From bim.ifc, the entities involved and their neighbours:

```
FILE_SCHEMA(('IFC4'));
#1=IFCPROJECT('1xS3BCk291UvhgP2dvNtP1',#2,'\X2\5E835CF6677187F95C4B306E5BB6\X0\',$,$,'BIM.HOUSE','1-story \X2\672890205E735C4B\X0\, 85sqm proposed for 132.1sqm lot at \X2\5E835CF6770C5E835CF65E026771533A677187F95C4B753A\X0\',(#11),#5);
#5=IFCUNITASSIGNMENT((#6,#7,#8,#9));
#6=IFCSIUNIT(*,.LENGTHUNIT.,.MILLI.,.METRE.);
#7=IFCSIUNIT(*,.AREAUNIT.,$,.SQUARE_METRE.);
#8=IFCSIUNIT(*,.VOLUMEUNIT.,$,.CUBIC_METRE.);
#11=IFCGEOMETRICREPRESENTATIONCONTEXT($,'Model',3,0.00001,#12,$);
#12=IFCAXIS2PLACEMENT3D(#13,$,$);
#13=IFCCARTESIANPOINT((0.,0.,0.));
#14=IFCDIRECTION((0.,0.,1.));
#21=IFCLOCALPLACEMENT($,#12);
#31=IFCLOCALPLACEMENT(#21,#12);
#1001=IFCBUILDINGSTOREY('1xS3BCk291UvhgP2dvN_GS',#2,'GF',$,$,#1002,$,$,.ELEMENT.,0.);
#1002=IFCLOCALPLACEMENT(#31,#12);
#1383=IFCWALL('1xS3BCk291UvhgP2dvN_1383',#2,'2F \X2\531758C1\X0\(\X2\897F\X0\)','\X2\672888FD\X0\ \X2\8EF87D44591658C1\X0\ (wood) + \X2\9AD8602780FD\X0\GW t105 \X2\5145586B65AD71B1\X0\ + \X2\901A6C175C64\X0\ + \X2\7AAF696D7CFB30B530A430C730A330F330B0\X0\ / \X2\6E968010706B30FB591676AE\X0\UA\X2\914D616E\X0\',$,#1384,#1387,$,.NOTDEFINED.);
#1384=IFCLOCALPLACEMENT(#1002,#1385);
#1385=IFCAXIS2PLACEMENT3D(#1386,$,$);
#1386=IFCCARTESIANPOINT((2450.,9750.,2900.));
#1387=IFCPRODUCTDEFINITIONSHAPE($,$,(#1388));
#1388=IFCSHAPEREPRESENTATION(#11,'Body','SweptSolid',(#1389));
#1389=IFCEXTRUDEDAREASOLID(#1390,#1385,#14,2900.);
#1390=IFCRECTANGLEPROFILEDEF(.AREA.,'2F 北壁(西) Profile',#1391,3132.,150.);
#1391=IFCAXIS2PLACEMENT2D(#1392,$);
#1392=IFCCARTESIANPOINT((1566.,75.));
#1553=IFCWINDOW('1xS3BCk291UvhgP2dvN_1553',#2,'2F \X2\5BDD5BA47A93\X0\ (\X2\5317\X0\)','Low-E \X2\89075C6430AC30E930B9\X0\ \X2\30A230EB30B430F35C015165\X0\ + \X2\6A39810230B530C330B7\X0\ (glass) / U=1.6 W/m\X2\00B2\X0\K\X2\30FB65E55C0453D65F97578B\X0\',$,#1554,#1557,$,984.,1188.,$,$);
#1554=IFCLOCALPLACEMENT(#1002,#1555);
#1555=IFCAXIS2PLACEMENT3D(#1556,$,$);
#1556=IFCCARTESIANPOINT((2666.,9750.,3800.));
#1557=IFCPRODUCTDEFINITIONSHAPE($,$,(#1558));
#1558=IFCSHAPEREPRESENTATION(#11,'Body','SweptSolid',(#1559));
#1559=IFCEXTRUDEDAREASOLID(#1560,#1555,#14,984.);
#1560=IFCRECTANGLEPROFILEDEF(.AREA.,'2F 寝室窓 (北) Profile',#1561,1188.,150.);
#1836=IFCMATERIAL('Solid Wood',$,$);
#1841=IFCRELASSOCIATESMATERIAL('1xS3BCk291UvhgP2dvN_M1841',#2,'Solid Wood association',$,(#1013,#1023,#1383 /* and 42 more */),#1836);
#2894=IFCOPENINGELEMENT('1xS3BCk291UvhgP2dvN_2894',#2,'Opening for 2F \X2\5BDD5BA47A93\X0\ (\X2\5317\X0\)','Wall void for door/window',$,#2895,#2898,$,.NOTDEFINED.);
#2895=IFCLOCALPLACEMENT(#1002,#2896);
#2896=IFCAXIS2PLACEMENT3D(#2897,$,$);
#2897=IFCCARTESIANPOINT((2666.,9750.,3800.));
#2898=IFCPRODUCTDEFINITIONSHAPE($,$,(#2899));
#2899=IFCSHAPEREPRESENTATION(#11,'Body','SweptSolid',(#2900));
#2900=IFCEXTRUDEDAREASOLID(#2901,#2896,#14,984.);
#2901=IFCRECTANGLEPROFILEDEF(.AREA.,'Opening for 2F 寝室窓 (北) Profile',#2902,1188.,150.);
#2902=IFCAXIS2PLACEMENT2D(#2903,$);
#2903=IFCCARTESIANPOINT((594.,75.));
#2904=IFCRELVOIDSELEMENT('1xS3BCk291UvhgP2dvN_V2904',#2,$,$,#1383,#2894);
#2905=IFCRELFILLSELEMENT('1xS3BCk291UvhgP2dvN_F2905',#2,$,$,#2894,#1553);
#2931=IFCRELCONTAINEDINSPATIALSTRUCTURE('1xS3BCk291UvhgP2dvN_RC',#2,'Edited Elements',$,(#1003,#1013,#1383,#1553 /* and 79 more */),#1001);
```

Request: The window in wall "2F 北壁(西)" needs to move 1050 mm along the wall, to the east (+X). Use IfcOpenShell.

```python
import ifcopenshell
import ifcopenshell.api.geometry
import ifcopenshell.util.placement
import ifcopenshell.util.unit

model = ifcopenshell.open("bim.ifc")
unit_scale = ifcopenshell.util.unit.calculate_unit_scale(model)

window = model.by_id(1553)
opening = window.FillsVoids[0].RelatingOpeningElement
wall = opening.VoidsElements[0].RelatingBuildingElement

wall_matrix = ifcopenshell.util.placement.get_local_placement(wall.ObjectPlacement)
shift = wall_matrix[:3, 0] * 1.05 / unit_scale
before = ifcopenshell.util.placement.get_local_placement(window.ObjectPlacement)[:3, 3].copy()

# The window is not placed relative to its opening, so move both.
for product in (opening, window):
    matrix = ifcopenshell.util.placement.get_local_placement(product.ObjectPlacement)
    matrix[:3, 3] += shift
    ifcopenshell.api.geometry.edit_object_placement(model, product=product, matrix=matrix, is_si=False)

after = ifcopenshell.util.placement.get_local_placement(window.ObjectPlacement)[:3, 3]
print("window moved by", (after - before).round(3) + 0.0)

model.write("bim_v2.ifc")
```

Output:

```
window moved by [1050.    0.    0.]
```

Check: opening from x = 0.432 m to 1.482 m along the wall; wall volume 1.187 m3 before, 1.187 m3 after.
